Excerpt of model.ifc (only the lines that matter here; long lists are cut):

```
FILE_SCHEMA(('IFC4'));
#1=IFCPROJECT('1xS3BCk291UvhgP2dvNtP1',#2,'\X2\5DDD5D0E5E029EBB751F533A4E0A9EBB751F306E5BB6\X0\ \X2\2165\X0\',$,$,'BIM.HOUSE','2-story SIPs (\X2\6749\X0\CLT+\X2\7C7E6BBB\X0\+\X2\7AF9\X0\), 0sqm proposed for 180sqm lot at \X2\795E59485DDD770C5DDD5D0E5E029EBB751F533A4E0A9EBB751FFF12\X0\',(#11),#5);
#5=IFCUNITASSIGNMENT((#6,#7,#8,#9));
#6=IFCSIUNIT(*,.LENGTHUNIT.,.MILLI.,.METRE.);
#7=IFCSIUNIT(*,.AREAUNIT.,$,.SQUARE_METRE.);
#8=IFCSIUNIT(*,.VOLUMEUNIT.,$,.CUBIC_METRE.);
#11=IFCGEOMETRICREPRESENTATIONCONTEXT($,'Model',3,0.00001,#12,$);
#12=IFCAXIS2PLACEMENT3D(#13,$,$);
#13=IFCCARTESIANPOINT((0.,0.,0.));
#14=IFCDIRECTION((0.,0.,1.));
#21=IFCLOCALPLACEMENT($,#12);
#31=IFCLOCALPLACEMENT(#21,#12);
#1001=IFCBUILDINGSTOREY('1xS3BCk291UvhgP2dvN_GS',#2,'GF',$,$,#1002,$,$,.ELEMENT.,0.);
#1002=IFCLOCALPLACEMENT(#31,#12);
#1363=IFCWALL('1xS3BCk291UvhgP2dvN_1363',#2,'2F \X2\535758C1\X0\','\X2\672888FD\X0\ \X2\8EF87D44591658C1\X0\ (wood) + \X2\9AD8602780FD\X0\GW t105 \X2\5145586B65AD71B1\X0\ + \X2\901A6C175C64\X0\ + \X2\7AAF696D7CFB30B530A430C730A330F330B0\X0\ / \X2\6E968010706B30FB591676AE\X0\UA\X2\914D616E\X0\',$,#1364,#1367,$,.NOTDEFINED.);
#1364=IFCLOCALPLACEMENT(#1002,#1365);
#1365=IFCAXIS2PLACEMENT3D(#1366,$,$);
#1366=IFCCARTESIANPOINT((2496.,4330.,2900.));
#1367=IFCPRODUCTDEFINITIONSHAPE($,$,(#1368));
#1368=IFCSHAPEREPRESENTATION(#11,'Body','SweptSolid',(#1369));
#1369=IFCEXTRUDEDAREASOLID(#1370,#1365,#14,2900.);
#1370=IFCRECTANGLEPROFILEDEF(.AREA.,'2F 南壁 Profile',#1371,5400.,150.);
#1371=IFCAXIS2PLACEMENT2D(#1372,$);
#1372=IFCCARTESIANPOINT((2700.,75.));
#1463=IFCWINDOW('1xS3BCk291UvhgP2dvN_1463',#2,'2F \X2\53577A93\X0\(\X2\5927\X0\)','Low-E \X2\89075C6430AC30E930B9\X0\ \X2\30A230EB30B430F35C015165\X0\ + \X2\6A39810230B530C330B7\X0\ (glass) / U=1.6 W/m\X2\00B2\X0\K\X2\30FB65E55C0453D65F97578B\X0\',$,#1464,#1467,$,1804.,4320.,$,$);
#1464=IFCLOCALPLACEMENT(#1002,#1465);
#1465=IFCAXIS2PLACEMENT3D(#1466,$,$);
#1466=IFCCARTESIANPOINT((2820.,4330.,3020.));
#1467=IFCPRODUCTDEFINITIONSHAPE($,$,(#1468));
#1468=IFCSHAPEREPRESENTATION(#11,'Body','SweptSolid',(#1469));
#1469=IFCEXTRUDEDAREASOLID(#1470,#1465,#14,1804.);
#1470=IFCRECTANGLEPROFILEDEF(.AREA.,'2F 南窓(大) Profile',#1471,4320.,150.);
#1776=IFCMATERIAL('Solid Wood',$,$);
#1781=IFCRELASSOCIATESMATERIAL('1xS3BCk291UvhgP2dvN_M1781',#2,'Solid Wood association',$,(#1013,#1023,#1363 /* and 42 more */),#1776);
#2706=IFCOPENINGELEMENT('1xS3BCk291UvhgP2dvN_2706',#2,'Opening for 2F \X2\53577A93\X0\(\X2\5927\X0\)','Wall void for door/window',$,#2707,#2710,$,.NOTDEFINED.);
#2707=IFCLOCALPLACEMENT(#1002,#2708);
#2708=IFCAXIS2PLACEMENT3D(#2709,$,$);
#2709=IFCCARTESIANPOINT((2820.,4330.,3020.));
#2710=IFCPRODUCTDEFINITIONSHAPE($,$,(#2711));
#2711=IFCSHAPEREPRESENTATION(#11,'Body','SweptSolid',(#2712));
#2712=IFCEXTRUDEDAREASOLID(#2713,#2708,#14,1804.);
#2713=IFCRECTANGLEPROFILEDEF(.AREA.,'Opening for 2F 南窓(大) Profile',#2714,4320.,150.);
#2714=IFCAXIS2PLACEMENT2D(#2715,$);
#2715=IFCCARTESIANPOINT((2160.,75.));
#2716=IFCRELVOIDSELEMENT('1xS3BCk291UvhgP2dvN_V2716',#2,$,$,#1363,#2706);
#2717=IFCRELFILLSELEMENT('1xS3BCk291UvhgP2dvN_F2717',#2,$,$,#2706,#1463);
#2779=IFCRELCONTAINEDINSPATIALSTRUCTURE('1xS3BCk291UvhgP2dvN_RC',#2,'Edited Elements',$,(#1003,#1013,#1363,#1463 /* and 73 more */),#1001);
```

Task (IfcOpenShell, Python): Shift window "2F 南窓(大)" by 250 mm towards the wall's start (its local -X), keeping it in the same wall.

```python
import ifcopenshell
import ifcopenshell.api.geometry
import ifcopenshell.util.placement
import ifcopenshell.util.unit

model = ifcopenshell.open("model.ifc")
unit_scale = ifcopenshell.util.unit.calculate_unit_scale(model)

window = model.by_guid("1xS3BCk291UvhgP2dvN_1463")
opening = window.FillsVoids[0].RelatingOpeningElement
wall = opening.VoidsElements[0].RelatingBuildingElement

wall_matrix = ifcopenshell.util.placement.get_local_placement(wall.ObjectPlacement)
shift = wall_matrix[:3, 0] * -0.25 / unit_scale
before = ifcopenshell.util.placement.get_local_placement(window.ObjectPlacement)[:3, 3].copy()

# The window is not placed relative to its opening, so move both.
for product in (opening, window):
    matrix = ifcopenshell.util.placement.get_local_placement(product.ObjectPlacement)
    matrix[:3, 3] += shift
    ifcopenshell.api.geometry.edit_object_placement(model, product=product, matrix=matrix, is_si=False)

after = ifcopenshell.util.placement.get_local_placement(window.ObjectPlacement)[:3, 3]
print("window moved by", (after - before).round(3) + 0.0)

model.write("model_rev.ifc")
```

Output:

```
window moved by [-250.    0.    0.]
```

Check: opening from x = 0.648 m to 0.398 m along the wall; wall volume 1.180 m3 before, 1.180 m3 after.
